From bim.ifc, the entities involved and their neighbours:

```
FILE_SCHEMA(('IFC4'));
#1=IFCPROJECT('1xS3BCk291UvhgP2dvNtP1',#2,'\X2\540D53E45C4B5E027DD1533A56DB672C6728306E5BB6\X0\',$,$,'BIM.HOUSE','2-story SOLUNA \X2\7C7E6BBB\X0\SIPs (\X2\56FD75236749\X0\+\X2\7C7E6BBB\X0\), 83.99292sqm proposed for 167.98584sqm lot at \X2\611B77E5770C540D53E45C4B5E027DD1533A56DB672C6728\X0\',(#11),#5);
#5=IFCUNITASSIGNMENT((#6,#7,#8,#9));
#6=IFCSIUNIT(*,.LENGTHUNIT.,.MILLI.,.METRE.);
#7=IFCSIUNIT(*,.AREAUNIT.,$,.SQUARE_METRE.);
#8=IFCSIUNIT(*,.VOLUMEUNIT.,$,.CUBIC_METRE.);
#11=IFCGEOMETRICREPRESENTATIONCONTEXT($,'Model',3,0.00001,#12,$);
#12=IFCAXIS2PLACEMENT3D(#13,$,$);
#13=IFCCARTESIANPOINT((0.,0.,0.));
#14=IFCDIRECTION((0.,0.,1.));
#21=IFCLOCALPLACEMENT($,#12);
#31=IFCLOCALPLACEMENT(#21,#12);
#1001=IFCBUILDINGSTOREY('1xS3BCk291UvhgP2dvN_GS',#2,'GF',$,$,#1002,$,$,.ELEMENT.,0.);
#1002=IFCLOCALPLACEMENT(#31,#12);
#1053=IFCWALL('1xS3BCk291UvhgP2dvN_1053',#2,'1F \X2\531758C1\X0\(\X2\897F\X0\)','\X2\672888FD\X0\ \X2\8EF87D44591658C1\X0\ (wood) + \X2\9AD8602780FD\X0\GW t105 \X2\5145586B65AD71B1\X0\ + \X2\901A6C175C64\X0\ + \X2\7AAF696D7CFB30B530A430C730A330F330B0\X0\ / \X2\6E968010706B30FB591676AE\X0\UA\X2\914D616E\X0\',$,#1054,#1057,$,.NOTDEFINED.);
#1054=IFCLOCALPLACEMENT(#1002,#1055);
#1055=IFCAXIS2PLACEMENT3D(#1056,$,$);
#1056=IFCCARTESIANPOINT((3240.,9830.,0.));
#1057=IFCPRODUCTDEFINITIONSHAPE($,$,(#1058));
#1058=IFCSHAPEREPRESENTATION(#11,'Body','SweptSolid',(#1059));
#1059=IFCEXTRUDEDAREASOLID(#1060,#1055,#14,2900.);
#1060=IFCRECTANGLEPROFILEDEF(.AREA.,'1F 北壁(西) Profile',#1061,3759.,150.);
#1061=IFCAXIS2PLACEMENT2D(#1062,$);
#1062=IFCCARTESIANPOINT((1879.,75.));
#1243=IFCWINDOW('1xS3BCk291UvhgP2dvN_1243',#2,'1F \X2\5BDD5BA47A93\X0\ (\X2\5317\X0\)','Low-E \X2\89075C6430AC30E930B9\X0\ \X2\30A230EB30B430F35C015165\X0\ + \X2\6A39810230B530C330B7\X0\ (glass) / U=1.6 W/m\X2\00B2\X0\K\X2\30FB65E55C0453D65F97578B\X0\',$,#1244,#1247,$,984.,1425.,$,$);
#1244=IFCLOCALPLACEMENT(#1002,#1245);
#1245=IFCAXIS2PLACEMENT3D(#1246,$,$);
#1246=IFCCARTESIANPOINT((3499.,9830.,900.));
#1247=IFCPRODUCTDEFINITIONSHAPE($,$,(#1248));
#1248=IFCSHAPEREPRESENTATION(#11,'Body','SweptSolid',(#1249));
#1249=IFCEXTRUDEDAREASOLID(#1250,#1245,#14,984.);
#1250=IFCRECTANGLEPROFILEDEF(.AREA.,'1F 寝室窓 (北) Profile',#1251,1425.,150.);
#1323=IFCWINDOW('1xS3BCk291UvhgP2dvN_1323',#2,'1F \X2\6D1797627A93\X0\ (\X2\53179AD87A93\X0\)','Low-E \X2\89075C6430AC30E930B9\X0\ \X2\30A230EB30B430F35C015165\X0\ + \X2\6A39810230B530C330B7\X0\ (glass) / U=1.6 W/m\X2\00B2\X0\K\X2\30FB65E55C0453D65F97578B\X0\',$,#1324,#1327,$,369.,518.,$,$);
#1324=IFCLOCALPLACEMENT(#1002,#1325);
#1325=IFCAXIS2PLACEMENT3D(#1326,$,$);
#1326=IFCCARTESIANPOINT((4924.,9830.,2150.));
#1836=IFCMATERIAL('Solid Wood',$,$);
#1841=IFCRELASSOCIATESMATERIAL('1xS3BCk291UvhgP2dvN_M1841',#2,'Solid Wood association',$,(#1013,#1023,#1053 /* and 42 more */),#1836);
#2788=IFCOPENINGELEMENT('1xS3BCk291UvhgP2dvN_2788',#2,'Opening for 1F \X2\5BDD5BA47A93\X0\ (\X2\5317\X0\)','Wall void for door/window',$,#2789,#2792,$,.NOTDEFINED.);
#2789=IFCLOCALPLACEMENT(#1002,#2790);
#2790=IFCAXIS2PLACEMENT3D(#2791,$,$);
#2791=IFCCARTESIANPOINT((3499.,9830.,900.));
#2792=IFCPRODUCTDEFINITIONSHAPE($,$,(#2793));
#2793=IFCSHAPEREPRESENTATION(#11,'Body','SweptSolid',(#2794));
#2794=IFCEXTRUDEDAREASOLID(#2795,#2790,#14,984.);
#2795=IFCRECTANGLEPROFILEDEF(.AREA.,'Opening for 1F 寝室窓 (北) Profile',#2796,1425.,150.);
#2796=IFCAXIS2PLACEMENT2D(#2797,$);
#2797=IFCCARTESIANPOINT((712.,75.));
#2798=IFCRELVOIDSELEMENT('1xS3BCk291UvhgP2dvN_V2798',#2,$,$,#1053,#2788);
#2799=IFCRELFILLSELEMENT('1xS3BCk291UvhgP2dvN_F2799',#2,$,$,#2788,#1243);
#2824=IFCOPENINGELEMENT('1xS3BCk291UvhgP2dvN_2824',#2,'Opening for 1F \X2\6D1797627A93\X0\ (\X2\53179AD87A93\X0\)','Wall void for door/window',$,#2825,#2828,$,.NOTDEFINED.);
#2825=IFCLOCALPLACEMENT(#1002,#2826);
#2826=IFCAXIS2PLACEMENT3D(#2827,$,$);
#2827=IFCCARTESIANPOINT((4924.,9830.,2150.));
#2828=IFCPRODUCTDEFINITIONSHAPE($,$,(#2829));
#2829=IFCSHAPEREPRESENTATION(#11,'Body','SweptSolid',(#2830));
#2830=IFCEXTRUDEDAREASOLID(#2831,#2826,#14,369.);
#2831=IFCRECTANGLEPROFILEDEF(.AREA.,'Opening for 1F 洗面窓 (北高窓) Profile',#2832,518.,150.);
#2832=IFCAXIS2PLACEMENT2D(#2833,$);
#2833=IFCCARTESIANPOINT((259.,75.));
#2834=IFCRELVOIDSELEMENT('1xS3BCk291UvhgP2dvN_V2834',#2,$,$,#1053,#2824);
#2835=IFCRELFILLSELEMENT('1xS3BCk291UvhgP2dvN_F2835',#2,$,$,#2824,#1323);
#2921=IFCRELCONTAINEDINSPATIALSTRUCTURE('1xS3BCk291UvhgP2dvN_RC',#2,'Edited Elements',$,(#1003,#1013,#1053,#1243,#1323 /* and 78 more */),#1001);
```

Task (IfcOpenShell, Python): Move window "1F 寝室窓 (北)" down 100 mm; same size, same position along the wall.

```python
import numpy as np
import ifcopenshell
import ifcopenshell.api.geometry
import ifcopenshell.util.placement
import ifcopenshell.util.unit

model = ifcopenshell.open("bim.ifc")
unit_scale = ifcopenshell.util.unit.calculate_unit_scale(model)

window = model.by_id(1243)
opening = window.FillsVoids[0].RelatingOpeningElement
dz = -0.1 / unit_scale

shift = np.array([0.0, 0.0, dz])
# The window is not placed relative to its opening, so move both.
for product in (opening, window):
    matrix = ifcopenshell.util.placement.get_local_placement(product.ObjectPlacement)
    matrix[:3, 3] += shift
    ifcopenshell.api.geometry.edit_object_placement(model, product=product, matrix=matrix, is_si=False)

print(f"moved by {dz * unit_scale:+.3f} m")

model.write("bim-out.ifc")
```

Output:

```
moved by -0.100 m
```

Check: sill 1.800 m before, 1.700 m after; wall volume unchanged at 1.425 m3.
